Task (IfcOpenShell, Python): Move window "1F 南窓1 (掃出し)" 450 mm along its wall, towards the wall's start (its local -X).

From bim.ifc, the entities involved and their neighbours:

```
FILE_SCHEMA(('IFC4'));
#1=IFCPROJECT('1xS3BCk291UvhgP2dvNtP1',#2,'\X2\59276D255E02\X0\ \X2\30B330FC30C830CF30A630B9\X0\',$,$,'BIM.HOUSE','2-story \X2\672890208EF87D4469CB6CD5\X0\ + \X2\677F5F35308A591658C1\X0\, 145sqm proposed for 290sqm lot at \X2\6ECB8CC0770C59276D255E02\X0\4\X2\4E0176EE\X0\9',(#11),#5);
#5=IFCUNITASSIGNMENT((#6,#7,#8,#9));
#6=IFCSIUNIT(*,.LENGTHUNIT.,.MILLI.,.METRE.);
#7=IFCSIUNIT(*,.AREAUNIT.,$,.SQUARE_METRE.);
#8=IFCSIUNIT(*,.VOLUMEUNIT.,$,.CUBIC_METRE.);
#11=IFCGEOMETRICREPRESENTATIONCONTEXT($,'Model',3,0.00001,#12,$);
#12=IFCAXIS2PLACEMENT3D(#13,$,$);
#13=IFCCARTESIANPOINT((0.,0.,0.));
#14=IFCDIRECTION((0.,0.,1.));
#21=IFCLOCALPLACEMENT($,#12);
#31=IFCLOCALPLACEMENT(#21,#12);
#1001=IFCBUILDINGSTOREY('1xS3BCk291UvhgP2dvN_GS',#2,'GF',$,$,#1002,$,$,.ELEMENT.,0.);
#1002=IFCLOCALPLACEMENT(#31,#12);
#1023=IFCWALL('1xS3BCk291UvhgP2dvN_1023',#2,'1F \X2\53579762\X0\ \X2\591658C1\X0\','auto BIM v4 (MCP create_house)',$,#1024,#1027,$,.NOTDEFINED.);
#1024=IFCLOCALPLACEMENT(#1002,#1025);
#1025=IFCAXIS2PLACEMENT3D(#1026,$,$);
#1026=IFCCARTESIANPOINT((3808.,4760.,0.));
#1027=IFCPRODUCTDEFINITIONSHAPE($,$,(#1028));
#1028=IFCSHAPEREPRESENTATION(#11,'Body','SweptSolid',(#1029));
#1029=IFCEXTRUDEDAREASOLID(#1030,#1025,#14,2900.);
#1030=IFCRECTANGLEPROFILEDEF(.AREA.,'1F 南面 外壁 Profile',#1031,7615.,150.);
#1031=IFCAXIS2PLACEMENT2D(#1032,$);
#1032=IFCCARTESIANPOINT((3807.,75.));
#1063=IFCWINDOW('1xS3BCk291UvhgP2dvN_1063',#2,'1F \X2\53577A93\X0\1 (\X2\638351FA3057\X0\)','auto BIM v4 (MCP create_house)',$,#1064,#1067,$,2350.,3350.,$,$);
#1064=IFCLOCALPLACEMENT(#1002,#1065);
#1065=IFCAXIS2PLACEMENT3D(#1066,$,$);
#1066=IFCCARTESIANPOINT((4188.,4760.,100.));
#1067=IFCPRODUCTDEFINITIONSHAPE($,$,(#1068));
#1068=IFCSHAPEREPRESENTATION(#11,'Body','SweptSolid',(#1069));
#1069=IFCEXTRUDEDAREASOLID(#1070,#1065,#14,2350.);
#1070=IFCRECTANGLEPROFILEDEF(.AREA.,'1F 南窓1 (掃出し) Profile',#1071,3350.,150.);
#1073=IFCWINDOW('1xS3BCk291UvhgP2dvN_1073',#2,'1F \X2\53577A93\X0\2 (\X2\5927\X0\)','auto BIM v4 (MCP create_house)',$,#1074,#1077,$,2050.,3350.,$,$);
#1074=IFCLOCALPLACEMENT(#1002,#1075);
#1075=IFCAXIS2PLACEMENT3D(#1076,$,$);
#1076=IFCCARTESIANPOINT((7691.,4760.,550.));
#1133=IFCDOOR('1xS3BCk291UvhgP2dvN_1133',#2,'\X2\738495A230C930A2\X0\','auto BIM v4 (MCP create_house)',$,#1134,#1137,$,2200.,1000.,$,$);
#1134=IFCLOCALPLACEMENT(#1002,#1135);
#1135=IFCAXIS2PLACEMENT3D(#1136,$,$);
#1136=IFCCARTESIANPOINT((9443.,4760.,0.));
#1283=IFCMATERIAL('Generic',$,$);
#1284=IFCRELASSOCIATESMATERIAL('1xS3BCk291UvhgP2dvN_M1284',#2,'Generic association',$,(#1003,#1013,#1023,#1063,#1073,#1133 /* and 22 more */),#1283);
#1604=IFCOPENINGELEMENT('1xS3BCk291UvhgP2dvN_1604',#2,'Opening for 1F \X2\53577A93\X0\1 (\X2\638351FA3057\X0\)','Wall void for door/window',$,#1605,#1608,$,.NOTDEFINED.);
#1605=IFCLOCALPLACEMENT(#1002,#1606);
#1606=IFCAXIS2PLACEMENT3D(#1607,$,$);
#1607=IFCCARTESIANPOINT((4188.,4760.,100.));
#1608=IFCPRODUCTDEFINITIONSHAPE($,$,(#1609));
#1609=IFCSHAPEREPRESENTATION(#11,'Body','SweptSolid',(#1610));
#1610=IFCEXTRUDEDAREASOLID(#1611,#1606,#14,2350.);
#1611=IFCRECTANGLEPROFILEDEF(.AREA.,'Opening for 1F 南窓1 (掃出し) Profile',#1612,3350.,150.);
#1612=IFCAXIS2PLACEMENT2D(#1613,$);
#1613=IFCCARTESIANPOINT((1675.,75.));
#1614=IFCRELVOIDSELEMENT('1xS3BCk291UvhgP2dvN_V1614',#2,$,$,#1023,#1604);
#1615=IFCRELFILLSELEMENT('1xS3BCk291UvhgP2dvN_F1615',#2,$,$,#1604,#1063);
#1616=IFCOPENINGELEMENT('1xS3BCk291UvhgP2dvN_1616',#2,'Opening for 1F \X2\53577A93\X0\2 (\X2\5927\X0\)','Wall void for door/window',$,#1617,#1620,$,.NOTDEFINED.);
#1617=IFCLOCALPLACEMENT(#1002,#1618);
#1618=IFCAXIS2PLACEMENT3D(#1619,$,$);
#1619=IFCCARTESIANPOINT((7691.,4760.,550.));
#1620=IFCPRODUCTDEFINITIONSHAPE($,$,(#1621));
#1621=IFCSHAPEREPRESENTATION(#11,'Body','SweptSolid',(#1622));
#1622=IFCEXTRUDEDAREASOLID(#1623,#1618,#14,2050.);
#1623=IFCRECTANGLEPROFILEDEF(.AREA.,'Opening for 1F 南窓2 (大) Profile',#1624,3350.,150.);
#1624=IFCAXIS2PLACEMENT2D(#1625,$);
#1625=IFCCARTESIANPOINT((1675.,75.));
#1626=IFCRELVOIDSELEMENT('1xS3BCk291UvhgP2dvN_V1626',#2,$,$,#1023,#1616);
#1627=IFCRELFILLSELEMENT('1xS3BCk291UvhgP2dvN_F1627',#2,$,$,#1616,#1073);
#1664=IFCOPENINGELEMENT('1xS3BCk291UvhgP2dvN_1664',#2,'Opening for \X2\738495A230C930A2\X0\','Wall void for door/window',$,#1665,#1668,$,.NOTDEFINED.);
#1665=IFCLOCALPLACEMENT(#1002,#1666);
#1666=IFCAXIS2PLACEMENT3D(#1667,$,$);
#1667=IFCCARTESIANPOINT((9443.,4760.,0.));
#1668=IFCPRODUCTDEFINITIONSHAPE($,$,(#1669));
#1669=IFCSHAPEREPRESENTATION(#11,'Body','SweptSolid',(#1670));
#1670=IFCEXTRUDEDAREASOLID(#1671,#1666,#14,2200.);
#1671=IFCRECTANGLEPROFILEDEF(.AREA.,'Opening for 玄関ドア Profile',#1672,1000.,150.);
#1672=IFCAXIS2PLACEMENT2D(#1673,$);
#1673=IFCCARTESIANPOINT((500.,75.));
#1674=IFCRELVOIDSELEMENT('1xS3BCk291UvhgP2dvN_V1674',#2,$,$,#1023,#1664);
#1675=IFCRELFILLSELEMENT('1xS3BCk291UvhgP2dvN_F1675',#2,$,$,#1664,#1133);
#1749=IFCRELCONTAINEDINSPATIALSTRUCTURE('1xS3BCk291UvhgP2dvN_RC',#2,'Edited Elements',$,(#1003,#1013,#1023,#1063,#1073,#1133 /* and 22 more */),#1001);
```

```python
import ifcopenshell
import ifcopenshell.api.geometry
import ifcopenshell.util.placement
import ifcopenshell.util.unit

model = ifcopenshell.open("bim.ifc")
unit_scale = ifcopenshell.util.unit.calculate_unit_scale(model)

window = model.by_guid("1xS3BCk291UvhgP2dvN_1063")
opening = window.FillsVoids[0].RelatingOpeningElement
wall = opening.VoidsElements[0].RelatingBuildingElement

wall_matrix = ifcopenshell.util.placement.get_local_placement(wall.ObjectPlacement)
shift = wall_matrix[:3, 0] * -0.45 / unit_scale
before = ifcopenshell.util.placement.get_local_placement(window.ObjectPlacement)[:3, 3].copy()

# The window is not placed relative to its opening, so move both.
for product in (opening, window):
    matrix = ifcopenshell.util.placement.get_local_placement(product.ObjectPlacement)
    matrix[:3, 3] += shift
    ifcopenshell.api.geometry.edit_object_placement(model, product=product, matrix=matrix, is_si=False)

after = ifcopenshell.util.placement.get_local_placement(window.ObjectPlacement)[:3, 3]
print("window moved by", (after - before).round(3) + 0.0)

model.write("bim_edited.ifc")
```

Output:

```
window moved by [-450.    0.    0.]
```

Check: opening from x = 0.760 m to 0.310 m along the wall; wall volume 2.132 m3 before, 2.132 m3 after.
